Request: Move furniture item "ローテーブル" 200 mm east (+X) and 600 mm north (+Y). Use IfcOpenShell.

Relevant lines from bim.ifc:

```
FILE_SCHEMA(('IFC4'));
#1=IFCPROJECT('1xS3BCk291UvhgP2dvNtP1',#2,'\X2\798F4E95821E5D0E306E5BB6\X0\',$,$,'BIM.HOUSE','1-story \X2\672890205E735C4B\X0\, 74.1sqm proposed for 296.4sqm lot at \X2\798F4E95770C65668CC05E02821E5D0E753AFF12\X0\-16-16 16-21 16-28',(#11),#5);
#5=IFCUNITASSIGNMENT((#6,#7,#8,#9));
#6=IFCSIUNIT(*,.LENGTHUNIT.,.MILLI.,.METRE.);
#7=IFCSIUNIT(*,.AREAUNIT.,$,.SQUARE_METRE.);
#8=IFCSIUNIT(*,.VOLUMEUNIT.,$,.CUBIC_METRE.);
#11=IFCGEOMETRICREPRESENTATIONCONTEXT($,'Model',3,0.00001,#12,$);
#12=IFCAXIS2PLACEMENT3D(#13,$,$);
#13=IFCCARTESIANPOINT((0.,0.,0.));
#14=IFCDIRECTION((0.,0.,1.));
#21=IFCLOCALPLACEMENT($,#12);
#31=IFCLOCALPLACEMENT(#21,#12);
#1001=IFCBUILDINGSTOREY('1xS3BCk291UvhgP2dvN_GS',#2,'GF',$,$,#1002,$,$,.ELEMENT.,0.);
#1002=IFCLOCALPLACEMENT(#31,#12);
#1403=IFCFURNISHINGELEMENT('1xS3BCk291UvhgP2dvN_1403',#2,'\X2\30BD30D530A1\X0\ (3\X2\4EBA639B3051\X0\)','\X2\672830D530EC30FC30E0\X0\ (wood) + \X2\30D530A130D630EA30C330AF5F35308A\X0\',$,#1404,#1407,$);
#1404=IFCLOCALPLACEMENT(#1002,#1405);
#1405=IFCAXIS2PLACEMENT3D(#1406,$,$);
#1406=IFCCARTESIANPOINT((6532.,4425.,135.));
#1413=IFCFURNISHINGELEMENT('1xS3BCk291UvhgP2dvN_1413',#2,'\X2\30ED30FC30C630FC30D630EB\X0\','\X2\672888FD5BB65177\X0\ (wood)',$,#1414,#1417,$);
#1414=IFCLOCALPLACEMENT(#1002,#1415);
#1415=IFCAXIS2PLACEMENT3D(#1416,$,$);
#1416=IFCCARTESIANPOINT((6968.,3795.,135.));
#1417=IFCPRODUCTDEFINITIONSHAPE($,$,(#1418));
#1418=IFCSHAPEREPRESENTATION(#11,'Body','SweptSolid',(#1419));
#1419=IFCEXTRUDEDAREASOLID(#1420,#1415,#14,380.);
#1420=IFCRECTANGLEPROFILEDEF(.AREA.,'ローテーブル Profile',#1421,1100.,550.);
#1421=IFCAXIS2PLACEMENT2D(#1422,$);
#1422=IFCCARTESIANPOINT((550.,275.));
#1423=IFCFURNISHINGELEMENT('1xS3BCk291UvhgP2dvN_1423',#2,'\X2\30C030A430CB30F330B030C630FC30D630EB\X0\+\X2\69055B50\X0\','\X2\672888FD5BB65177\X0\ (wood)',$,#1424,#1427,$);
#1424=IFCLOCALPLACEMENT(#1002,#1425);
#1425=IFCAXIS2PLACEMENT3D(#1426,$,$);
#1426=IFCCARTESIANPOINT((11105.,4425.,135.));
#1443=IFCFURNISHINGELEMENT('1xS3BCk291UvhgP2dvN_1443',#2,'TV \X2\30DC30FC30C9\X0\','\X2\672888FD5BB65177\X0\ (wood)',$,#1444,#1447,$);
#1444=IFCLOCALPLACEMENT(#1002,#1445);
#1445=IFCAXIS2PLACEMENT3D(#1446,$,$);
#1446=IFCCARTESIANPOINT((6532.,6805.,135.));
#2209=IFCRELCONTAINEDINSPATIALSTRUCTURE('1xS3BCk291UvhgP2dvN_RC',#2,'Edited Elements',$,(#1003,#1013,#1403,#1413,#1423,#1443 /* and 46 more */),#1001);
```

```python
import ifcopenshell
import ifcopenshell.api.geometry
import ifcopenshell.util.placement
import ifcopenshell.util.unit

model = ifcopenshell.open("bim.ifc")
unit_scale = ifcopenshell.util.unit.calculate_unit_scale(model)

item = model.by_guid("1xS3BCk291UvhgP2dvN_1413")
matrix = ifcopenshell.util.placement.get_local_placement(item.ObjectPlacement)
matrix[0, 3] += 0.2 / unit_scale
matrix[1, 3] += 0.6 / unit_scale
ifcopenshell.api.geometry.edit_object_placement(model, product=item, matrix=matrix, is_si=False)

print(ifcopenshell.util.placement.get_local_placement(item.ObjectPlacement).round(3) + 0.0)

model.write("bim-out.ifc")
```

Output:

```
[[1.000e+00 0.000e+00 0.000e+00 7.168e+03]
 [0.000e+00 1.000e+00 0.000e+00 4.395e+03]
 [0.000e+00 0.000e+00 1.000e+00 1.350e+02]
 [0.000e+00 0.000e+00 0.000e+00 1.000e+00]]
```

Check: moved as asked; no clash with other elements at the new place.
